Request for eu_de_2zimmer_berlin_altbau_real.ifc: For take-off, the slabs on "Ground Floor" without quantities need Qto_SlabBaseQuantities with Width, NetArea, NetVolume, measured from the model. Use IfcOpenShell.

First a look at what the model holds.

```python
import ifcopenshell
import ifcopenshell.util.element
import ifcopenshell.util.unit

model = ifcopenshell.open("eu_de_2zimmer_berlin_altbau_real.ifc")
print(model.schema)
for unit_type in ("LENGTHUNIT", "AREAUNIT", "VOLUMEUNIT"):
    print(unit_type, ifcopenshell.util.unit.calculate_unit_scale(model, unit_type))
storey = next(s for s in model.by_type("IfcBuildingStorey") if s.Name == "Ground Floor")
slabs = [e for e in ifcopenshell.util.element.get_decomposition(storey) if e.is_a("IfcSlab")]
for e in sorted(slabs, key=lambda e: e.id()):
    print(e.id(), e.is_a(), e.Name, list(ifcopenshell.util.element.get_psets(e, qtos_only=True)), sep=" | ")
```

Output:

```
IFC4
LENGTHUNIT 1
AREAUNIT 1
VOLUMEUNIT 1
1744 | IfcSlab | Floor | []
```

```python
import ifcopenshell
import ifcopenshell.api.pset
import ifcopenshell.geom
import ifcopenshell.util.element
import ifcopenshell.util.shape
import ifcopenshell.util.unit

model = ifcopenshell.open("eu_de_2zimmer_berlin_altbau_real.ifc")
unit_scale = ifcopenshell.util.unit.calculate_unit_scale(model)
area_scale = ifcopenshell.util.unit.calculate_unit_scale(model, "AREAUNIT")
volume_scale = ifcopenshell.util.unit.calculate_unit_scale(model, "VOLUMEUNIT")
settings = ifcopenshell.geom.settings()

storey = next(s for s in model.by_type("IfcBuildingStorey") if s.Name == "Ground Floor")
slabs = [e for e in ifcopenshell.util.element.get_decomposition(storey) if e.is_a("IfcSlab")]

for e in sorted(slabs, key=lambda e: e.id()):
    if ifcopenshell.util.element.get_psets(e, qtos_only=True, should_inherit=False):
        continue
    # Geometry comes back in metres, in the element's own axes.
    shape = ifcopenshell.geom.create_shape(settings, e)
    values = {
        "Width": ifcopenshell.util.shape.get_z(shape.geometry) / unit_scale,
        "NetArea": ifcopenshell.util.shape.get_footprint_area(shape.geometry) / area_scale,
        "NetVolume": ifcopenshell.util.shape.get_volume(shape.geometry) / volume_scale,
    }
    qto = ifcopenshell.api.pset.add_qto(model, product=e, name="Qto_SlabBaseQuantities")
    ifcopenshell.api.pset.edit_qto(model, qto=qto, properties=values)
    print(e.id(), {k: round(v, 3) for k, v in values.items()})

model.write("eu_de_2zimmer_berlin_altbau_real_edited.ifc")
```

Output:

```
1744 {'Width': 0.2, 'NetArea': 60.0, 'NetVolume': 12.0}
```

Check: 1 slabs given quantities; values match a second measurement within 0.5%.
